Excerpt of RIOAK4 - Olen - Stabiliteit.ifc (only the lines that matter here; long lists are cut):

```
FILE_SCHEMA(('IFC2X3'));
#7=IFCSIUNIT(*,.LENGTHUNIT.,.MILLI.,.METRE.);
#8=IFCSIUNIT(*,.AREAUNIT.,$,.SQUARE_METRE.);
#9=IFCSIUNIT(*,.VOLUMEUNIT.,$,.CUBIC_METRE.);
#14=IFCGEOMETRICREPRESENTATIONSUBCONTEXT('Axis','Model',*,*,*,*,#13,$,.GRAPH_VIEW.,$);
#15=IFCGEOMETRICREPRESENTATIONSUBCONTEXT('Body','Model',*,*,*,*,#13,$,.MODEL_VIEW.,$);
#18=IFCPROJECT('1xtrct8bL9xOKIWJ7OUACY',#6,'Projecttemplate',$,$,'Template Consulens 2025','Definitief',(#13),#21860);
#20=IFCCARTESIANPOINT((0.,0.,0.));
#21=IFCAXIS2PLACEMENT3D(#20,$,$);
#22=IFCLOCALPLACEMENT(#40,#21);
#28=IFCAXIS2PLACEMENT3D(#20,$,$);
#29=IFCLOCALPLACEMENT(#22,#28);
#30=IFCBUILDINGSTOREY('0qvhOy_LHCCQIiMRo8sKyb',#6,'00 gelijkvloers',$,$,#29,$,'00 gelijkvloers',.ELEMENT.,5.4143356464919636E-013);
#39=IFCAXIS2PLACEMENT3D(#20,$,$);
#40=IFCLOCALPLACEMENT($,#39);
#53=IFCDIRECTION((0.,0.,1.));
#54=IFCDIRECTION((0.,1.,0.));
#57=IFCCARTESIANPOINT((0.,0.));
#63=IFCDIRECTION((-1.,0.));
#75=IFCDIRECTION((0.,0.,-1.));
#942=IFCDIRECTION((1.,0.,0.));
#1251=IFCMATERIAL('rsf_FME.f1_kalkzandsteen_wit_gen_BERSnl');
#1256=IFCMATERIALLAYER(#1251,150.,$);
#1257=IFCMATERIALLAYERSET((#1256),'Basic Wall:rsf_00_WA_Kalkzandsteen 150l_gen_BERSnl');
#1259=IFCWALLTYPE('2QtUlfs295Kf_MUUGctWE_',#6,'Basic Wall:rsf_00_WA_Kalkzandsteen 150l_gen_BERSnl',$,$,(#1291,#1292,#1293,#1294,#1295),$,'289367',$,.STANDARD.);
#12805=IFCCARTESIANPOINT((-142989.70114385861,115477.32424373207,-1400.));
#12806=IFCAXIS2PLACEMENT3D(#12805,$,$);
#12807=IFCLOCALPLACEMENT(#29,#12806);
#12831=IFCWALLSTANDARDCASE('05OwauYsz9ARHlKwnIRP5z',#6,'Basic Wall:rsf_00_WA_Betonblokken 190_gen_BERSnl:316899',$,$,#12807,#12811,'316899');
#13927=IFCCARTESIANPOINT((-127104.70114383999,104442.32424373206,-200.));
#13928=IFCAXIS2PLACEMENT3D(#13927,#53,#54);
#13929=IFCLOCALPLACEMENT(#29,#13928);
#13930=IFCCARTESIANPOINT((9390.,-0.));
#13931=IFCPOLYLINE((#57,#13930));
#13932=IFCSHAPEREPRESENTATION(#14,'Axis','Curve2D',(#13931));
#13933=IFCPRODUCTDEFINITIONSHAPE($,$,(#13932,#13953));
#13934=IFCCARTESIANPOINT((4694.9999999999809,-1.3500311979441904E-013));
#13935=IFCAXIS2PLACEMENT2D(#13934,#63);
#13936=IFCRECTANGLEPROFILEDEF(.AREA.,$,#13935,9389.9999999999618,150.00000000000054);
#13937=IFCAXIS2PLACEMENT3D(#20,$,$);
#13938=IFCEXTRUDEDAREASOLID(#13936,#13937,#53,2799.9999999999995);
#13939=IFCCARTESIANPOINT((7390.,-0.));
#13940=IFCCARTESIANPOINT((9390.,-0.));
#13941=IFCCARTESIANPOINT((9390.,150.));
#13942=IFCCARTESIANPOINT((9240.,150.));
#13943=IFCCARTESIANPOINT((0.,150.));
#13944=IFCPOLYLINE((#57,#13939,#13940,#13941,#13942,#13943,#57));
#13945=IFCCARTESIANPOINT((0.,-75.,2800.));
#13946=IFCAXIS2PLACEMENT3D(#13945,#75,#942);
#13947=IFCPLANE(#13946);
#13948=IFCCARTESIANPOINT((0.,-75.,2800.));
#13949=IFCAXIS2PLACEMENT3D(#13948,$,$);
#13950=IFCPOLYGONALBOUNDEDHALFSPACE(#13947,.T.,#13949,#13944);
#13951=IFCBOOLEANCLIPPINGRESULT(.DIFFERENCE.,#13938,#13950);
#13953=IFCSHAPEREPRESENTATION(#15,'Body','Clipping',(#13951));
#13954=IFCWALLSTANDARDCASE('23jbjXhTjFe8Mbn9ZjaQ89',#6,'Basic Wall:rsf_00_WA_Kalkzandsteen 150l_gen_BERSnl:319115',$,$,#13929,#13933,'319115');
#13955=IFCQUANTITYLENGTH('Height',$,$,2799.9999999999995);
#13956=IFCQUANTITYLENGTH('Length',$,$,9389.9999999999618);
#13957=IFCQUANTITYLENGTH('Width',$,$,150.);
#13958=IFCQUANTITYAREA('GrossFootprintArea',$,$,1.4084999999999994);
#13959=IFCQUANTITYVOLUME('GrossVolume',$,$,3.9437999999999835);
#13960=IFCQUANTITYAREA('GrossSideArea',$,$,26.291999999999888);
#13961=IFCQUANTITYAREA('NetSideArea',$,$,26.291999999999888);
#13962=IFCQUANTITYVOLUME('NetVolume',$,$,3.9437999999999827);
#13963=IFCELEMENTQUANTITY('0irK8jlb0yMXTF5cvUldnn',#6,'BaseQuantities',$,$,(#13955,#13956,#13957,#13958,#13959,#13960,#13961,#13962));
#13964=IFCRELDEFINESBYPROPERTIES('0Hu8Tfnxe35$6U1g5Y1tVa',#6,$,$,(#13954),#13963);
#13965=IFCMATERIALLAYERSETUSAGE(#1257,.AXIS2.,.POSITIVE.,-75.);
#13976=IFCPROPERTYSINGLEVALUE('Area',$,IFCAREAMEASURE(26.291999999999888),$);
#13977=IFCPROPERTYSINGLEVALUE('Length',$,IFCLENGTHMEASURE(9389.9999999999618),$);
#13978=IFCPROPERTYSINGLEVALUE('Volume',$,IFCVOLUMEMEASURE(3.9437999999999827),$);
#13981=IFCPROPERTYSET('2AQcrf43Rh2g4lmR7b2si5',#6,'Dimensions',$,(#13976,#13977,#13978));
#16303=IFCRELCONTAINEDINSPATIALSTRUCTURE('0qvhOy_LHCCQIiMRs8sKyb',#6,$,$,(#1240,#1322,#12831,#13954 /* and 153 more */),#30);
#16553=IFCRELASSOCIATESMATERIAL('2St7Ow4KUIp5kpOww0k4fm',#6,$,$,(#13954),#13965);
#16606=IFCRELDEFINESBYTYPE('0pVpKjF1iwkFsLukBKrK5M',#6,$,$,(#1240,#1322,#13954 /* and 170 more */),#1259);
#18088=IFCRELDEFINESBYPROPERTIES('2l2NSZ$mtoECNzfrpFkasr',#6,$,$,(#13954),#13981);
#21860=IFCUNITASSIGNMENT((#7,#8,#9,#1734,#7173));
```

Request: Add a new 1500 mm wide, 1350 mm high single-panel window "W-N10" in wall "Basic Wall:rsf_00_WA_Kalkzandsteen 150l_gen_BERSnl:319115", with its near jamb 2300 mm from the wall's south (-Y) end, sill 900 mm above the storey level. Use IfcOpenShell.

```python
import numpy as np
import ifcopenshell
import ifcopenshell.api.feature
import ifcopenshell.api.geometry
import ifcopenshell.api.pset
import ifcopenshell.api.root
import ifcopenshell.api.spatial
import ifcopenshell.api.type
import ifcopenshell.geom
import ifcopenshell.util.element
import ifcopenshell.util.placement
import ifcopenshell.util.representation
import ifcopenshell.util.shape
import ifcopenshell.util.unit

model = ifcopenshell.open("RIOAK4 - Olen - Stabiliteit.ifc")
unit_scale = ifcopenshell.util.unit.calculate_unit_scale(model)
area_scale = ifcopenshell.util.unit.calculate_unit_scale(model, "AREAUNIT")
volume_scale = ifcopenshell.util.unit.calculate_unit_scale(model, "VOLUMEUNIT")
settings = ifcopenshell.geom.settings()


def volume(element):
    """Net volume in cubic metres, openings subtracted."""
    shape = ifcopenshell.geom.create_shape(settings, element)
    return ifcopenshell.util.shape.get_volume(shape.geometry)


wall = model.by_guid("23jbjXhTjFe8Mbn9ZjaQ89")
storey = ifcopenshell.util.element.get_container(wall, ifc_class="IfcBuildingStorey")
context = ifcopenshell.util.representation.get_context(model, "Model", "Body", "MODEL_VIEW")
before = volume(wall)

width, height, from_end, sill = 1.5, 1.35, 2.3, 0.9  # metres

# The wall runs along its own X axis, and the end named is its -X end.
wall_shape = ifcopenshell.geom.create_shape(settings, wall)
x, y, z = ifcopenshell.util.shape.get_vertices(wall_shape.geometry).T
start = x.min() + from_end
face, thickness = float(y.min()), float(y.max() - y.min())
wall_matrix = ifcopenshell.util.placement.get_local_placement(wall.ObjectPlacement)
level = ifcopenshell.util.placement.get_local_placement(storey.ObjectPlacement)[2, 3]


def in_wall(x, y):
    """Placement at x, y metres in the wall's axes, at sill height."""
    matrix = wall_matrix.copy()
    matrix[:, 3] = wall_matrix @ np.array([x / unit_scale, y / unit_scale, 0.0, 1.0])
    matrix[2, 3] = level + sill / unit_scale
    return matrix


# Opening: a box that overshoots both wall faces by 50 mm.
opening = ifcopenshell.api.root.create_entity(model, ifc_class="IfcOpeningElement")
box = ifcopenshell.api.geometry.add_wall_representation(
    model, context=context, length=width, height=height, thickness=thickness + 0.1
)
ifcopenshell.api.geometry.assign_representation(model, product=opening, representation=box)
ifcopenshell.api.geometry.edit_object_placement(model, product=opening, matrix=in_wall(start, face - 0.05), is_si=False)
ifcopenshell.api.feature.add_feature(model, feature=opening, element=wall)

window = ifcopenshell.api.root.create_entity(model, ifc_class="IfcWindow", name="W-N10")
window.OverallWidth, window.OverallHeight = width / unit_scale, height / unit_scale
body = ifcopenshell.api.geometry.add_window_representation(
    model,
    context=context,
    overall_width=window.OverallWidth,
    overall_height=window.OverallHeight,
    partition_type="SINGLE_PANEL",
)
ifcopenshell.api.geometry.assign_representation(model, product=window, representation=body)
ifcopenshell.api.spatial.assign_container(model, products=[window], relating_structure=storey)
fills = ifcopenshell.api.feature.add_filling(model, opening=opening, element=window)
fills.OwnerHistory = window.OwnerHistory  # required in IFC2X3

# IFC2X3 keeps the operation on the window style.
style = ifcopenshell.api.root.create_entity(model, ifc_class="IfcWindowStyle", name="W-N10")
style.OperationType, style.ConstructionType = "SINGLE_PANEL", "NOTDEFINED"
style.ParameterTakesPrecedence = style.Sizeable = False
ifcopenshell.api.type.assign_type(model, related_objects=[window], relating_type=style)

# Centre the window in the wall's thickness.
ifcopenshell.api.geometry.edit_object_placement(model, product=window, matrix=in_wall(start, face), is_si=False)
window_shape = ifcopenshell.geom.create_shape(settings, window)
depth = ifcopenshell.util.shape.get_vertices(window_shape.geometry)[:, 1]
offset = face + thickness / 2 - (depth.min() + depth.max()) / 2
ifcopenshell.api.geometry.edit_object_placement(model, product=window, matrix=in_wall(start, offset), is_si=False)

after = volume(wall)

# Update the wall's stored quantities.
qto = model.by_id(ifcopenshell.util.element.get_pset(wall, "BaseQuantities", should_inherit=False)["id"])
ifcopenshell.api.pset.edit_qto(model, qto=qto, properties={
    "NetSideArea": after / thickness / area_scale,
    "NetVolume": after / volume_scale,
})
pset = model.by_id(ifcopenshell.util.element.get_pset(wall, "Dimensions", should_inherit=False)["id"])
ifcopenshell.api.pset.edit_pset(model, pset=pset, properties={
    "Area": model.create_entity("IfcAreaMeasure", after / thickness / area_scale),
    "Volume": model.create_entity("IfcVolumeMeasure", after / volume_scale),
})

print(f"wall volume {before:.3f} -> {after:.3f} m3")

model.write("RIOAK4 - Olen - Stabiliteit_v2.ifc")
```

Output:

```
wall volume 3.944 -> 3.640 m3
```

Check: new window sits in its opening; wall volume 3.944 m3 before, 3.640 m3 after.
